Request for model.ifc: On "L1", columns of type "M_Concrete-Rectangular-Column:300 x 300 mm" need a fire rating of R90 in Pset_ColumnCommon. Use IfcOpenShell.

First a look at what the model holds.

```python
import ifcopenshell
import ifcopenshell.util.element

model = ifcopenshell.open("model.ifc")
print(model.schema)
storey = next(s for s in model.by_type("IfcBuildingStorey") if s.Name == "L1")
columns = [e for e in ifcopenshell.util.element.get_decomposition(storey) if e.is_a("IfcColumn")]
seen = {}
for e in columns:
    element_type = ifcopenshell.util.element.get_type(e)
    key = (element_type.Name if element_type != e and element_type else None, ifcopenshell.util.element.get_pset(e, "Pset_ColumnCommon", "FireRating"))
    seen[key] = seen.get(key, 0) + 1
for (name, value), count in sorted(seen.items(), key=str):
    print(count, "x", name, "|", value)
```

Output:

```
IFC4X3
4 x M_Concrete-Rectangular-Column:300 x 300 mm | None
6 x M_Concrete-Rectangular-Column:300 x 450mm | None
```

```python
import ifcopenshell
import ifcopenshell.api.pset
import ifcopenshell.util.element

model = ifcopenshell.open("model.ifc")

storey = next(s for s in model.by_type("IfcBuildingStorey") if s.Name == "L1")
columns = [e for e in ifcopenshell.util.element.get_decomposition(storey) if e.is_a("IfcColumn")]

count = 0
for e in columns:
    element_type = ifcopenshell.util.element.get_type(e)
    if element_type in (None, e) or element_type.Name != "M_Concrete-Rectangular-Column:300 x 300 mm":
        continue
    # add_pset returns the element's existing set when there is one.
    pset = ifcopenshell.api.pset.add_pset(model, product=e, name="Pset_ColumnCommon")
    ifcopenshell.api.pset.edit_pset(model, pset=pset, properties={"FireRating": "R90"})
    count += 1

print(count, "columns updated")

model.write("model_edited.ifc")
```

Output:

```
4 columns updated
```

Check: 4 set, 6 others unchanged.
